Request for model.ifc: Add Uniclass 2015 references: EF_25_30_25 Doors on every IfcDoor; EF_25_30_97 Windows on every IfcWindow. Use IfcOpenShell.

First a look at what the model holds.

```python
import ifcopenshell

model = ifcopenshell.open("model.ifc")
print(model.schema)
print("classifications:", [c.Name for c in model.by_type("IfcClassification")])
for ifc_class in ("IfcDoor", "IfcRoof", "IfcStair", "IfcWall", "IfcWindow"):
    print(ifc_class, len(model.by_type(ifc_class)))
```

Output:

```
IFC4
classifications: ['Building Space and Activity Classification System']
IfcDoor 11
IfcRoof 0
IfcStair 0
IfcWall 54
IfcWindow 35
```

```python
import ifcopenshell
import ifcopenshell.api.classification

model = ifcopenshell.open("model.ifc")

system = ifcopenshell.api.classification.add_classification(model, classification="Uniclass 2015")

codes = {
    "IfcDoor": ("EF_25_30_25", "Doors"),
    "IfcWindow": ("EF_25_30_97", "Windows"),
}
for ifc_class, (code, name) in codes.items():
    products = model.by_type(ifc_class)
    ifcopenshell.api.classification.add_reference(
        model, products=products, classification=system, identification=code, name=name
    )
    print(code, len(products))

model.write("model_edited.ifc")
```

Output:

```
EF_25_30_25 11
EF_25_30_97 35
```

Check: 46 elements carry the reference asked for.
